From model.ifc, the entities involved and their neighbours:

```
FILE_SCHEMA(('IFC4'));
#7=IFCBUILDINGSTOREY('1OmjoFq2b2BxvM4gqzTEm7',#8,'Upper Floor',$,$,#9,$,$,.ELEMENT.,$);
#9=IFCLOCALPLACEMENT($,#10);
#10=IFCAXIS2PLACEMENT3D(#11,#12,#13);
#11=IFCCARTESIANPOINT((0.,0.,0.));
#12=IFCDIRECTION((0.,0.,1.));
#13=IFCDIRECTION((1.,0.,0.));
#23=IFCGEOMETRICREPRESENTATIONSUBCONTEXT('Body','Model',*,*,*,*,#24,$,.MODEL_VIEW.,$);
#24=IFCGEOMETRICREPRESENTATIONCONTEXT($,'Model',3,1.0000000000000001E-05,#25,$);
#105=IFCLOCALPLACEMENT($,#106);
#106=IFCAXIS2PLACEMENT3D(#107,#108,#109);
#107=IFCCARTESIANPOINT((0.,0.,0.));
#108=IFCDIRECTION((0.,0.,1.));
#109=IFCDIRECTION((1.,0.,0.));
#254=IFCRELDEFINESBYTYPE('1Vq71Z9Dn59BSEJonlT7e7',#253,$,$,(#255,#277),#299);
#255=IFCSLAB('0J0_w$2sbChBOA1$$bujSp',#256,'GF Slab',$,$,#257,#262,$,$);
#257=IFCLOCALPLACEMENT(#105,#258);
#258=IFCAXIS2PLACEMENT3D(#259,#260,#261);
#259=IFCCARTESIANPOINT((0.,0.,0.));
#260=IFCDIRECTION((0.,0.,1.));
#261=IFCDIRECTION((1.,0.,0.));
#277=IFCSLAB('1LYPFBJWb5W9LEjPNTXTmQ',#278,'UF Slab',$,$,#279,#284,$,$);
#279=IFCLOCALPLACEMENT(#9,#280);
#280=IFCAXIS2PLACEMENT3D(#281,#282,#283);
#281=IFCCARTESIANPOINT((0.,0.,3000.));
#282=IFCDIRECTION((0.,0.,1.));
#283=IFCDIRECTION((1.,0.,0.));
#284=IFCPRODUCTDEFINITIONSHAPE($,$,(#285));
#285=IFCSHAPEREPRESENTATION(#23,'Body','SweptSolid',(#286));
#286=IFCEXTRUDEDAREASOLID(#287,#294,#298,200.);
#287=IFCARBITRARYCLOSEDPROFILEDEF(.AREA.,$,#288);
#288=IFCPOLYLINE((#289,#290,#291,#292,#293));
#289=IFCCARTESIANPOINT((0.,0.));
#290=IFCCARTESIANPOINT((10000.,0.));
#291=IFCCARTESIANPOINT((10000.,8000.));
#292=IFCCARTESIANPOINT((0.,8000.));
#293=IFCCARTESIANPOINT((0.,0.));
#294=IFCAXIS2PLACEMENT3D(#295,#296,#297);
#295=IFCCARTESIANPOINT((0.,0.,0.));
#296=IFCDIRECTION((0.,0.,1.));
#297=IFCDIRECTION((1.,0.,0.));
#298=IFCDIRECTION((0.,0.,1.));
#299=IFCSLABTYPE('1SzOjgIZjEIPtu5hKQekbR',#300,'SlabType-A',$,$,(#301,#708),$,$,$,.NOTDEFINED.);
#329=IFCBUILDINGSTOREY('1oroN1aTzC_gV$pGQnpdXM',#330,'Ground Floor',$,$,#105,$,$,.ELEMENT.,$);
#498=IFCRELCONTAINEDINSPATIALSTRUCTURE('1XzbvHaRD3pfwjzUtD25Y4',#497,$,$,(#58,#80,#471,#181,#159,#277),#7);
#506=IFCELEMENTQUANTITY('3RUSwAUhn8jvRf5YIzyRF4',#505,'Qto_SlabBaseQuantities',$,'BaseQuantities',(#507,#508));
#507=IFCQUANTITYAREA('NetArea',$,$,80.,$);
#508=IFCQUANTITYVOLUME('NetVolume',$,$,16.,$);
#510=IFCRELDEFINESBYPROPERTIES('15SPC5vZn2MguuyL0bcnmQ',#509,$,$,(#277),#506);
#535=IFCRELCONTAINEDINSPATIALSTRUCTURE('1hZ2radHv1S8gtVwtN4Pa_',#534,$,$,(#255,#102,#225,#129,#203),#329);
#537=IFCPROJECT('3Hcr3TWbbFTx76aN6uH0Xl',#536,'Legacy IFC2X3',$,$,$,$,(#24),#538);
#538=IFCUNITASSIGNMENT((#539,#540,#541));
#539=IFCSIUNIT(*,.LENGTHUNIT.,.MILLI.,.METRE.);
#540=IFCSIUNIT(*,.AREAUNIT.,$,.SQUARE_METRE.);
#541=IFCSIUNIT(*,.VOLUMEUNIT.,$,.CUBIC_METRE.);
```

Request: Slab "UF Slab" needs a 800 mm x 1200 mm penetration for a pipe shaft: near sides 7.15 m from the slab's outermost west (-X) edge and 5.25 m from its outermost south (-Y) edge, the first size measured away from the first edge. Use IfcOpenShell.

```python
import numpy as np
import ifcopenshell
import ifcopenshell.api.feature
import ifcopenshell.api.geometry
import ifcopenshell.api.pset
import ifcopenshell.api.root
import ifcopenshell.geom
import ifcopenshell.util.element
import ifcopenshell.util.placement
import ifcopenshell.util.representation
import ifcopenshell.util.shape
import ifcopenshell.util.unit

model = ifcopenshell.open("model.ifc")
unit_scale = ifcopenshell.util.unit.calculate_unit_scale(model)
area_scale = ifcopenshell.util.unit.calculate_unit_scale(model, "AREAUNIT")
volume_scale = ifcopenshell.util.unit.calculate_unit_scale(model, "VOLUMEUNIT")
settings = ifcopenshell.geom.settings()


def volume(element):
    """Net volume in cubic metres, openings subtracted."""
    shape = ifcopenshell.geom.create_shape(settings, element)
    return ifcopenshell.util.shape.get_volume(shape.geometry)


slab = model.by_guid("1LYPFBJWb5W9LEjPNTXTmQ")
before = volume(slab)

# Extent in the slab's own axes, in metres. The edges named are its -X and -Y sides.
slab_shape = ifcopenshell.geom.create_shape(settings, slab)
vertices = ifcopenshell.util.shape.get_vertices(slab_shape.geometry)
x_min, y_min, bottom = vertices.min(axis=0)
top = vertices[:, 2].max()

opening = ifcopenshell.api.root.create_entity(model, ifc_class="IfcOpeningElement", name="Pipe shaft opening", predefined_type="OPENING")
context = ifcopenshell.util.representation.get_context(model, "Model", "Body", "MODEL_VIEW")
width, depth = 0.8, 1.2
outline = [(0.0, 0.0), (width, 0.0), (width, depth), (0.0, depth), (0.0, 0.0)]
# Overshoot both faces by 50 mm so the cut is clean.
shape = ifcopenshell.api.geometry.add_slab_representation(
    model, context=context, depth=top - bottom + 0.1, polyline=outline
)
ifcopenshell.api.geometry.assign_representation(model, product=opening, representation=shape)

matrix = ifcopenshell.util.placement.get_local_placement(slab.ObjectPlacement)
matrix[:, 3] = matrix @ np.append(np.array([x_min + 7.15, y_min + 5.25, bottom - 0.05]) / unit_scale, 1.0)
ifcopenshell.api.geometry.edit_object_placement(model, product=opening, matrix=matrix, is_si=False)
ifcopenshell.api.feature.add_feature(model, feature=opening, element=slab)

after = volume(slab)

# Update the slab's stored quantities.
qto = model.by_id(ifcopenshell.util.element.get_pset(slab, "Qto_SlabBaseQuantities", should_inherit=False)["id"])
ifcopenshell.api.pset.edit_qto(model, qto=qto, properties={
    "NetArea": after / (top - bottom) / area_scale,
    "NetVolume": after / volume_scale,
})

print(f"slab volume {before:.3f} -> {after:.3f} m3")

model.write("model_updated.ifc")
```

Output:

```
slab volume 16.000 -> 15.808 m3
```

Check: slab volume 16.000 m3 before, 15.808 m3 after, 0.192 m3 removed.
